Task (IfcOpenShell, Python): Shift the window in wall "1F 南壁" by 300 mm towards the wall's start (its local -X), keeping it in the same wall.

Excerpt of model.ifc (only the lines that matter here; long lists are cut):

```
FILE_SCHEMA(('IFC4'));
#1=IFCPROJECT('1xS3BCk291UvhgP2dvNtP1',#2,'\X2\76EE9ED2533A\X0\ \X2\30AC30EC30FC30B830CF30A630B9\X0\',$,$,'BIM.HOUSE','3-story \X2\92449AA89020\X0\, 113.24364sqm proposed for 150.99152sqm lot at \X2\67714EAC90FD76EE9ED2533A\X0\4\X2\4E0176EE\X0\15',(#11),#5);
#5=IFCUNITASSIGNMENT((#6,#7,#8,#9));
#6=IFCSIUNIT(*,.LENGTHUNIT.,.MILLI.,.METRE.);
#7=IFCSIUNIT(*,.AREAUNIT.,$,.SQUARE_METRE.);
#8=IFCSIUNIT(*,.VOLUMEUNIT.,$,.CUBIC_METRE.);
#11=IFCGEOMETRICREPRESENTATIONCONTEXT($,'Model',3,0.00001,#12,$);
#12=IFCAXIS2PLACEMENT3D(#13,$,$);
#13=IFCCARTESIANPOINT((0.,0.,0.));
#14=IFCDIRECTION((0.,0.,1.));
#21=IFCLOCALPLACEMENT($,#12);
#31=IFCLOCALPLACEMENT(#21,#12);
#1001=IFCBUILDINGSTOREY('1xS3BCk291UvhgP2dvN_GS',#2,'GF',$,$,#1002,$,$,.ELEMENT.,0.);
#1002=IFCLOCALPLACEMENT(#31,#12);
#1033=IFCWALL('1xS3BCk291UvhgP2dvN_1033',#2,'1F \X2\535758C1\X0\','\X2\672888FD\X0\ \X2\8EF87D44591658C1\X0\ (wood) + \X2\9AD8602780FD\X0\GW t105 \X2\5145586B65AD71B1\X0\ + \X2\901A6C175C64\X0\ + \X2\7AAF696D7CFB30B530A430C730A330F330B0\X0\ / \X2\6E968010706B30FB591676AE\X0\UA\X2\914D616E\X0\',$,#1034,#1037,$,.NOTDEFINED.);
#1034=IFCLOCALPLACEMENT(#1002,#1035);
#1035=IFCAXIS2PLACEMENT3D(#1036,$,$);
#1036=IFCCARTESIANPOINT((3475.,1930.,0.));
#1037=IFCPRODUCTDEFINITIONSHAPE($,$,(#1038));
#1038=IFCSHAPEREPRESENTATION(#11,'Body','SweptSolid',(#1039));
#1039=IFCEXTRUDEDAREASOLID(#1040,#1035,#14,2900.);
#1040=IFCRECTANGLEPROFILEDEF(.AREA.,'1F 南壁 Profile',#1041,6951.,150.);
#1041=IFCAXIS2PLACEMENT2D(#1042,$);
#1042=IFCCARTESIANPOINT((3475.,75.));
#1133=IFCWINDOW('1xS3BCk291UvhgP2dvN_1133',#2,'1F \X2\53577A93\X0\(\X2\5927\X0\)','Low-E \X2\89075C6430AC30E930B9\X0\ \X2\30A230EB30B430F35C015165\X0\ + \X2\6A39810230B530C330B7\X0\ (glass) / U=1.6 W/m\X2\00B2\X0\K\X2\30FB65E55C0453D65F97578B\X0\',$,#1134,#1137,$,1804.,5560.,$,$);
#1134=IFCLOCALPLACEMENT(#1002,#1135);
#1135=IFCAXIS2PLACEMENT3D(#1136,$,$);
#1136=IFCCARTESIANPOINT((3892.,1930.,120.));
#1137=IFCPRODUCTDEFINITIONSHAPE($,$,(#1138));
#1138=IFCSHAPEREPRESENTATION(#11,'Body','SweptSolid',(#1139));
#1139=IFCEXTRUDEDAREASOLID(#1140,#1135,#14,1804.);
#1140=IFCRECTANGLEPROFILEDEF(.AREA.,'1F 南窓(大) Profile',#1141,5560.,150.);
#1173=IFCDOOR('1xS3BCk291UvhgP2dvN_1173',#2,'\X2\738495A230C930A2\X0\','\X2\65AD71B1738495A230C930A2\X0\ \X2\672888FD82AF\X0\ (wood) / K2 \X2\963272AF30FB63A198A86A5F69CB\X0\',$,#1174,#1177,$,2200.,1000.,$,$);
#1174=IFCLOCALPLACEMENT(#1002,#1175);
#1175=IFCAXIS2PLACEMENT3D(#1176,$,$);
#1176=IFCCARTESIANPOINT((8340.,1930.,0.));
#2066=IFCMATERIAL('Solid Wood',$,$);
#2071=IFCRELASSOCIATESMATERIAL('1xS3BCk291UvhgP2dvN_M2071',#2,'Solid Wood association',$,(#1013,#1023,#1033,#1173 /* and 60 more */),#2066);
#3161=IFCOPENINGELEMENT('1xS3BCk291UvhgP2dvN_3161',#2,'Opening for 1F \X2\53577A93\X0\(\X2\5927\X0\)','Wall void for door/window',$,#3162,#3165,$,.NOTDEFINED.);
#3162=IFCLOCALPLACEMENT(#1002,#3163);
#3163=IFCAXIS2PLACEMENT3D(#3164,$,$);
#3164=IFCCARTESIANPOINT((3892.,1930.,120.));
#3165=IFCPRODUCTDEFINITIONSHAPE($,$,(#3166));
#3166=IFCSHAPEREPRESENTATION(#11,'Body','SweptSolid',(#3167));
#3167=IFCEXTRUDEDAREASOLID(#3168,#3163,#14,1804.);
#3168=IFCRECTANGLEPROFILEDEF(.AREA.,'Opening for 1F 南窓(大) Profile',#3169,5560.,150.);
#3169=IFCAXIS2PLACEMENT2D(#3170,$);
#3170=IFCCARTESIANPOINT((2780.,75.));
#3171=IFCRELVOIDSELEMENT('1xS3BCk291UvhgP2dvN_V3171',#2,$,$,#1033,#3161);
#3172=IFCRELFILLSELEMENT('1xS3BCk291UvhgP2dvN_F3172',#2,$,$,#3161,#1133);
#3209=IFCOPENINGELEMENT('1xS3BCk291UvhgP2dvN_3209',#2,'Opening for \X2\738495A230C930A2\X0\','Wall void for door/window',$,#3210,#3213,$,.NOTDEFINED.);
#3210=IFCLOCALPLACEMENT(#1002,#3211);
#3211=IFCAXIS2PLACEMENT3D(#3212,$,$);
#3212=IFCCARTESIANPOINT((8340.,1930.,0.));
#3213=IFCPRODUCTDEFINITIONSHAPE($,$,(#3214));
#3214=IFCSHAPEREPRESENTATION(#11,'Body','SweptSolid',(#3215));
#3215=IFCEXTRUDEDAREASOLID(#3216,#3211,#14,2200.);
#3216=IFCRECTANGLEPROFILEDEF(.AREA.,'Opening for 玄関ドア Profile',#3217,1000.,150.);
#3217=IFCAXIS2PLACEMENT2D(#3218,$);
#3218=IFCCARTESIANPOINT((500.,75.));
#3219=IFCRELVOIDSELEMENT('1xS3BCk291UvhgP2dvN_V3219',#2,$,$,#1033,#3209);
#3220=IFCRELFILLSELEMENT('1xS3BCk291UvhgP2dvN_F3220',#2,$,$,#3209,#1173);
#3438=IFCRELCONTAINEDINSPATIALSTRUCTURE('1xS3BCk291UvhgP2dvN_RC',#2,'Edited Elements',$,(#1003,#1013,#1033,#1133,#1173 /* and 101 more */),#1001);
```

```python
import ifcopenshell
import ifcopenshell.api.geometry
import ifcopenshell.util.placement
import ifcopenshell.util.unit

model = ifcopenshell.open("model.ifc")
unit_scale = ifcopenshell.util.unit.calculate_unit_scale(model)

window = model.by_guid("1xS3BCk291UvhgP2dvN_1133")
opening = window.FillsVoids[0].RelatingOpeningElement
wall = opening.VoidsElements[0].RelatingBuildingElement

wall_matrix = ifcopenshell.util.placement.get_local_placement(wall.ObjectPlacement)
shift = wall_matrix[:3, 0] * -0.3 / unit_scale
before = ifcopenshell.util.placement.get_local_placement(window.ObjectPlacement)[:3, 3].copy()

# The window is not placed relative to its opening, so move both.
for product in (opening, window):
    matrix = ifcopenshell.util.placement.get_local_placement(product.ObjectPlacement)
    matrix[:3, 3] += shift
    ifcopenshell.api.geometry.edit_object_placement(model, product=product, matrix=matrix, is_si=False)

after = ifcopenshell.util.placement.get_local_placement(window.ObjectPlacement)[:3, 3]
print("window moved by", (after - before).round(3) + 0.0)

model.write("model_rev.ifc")
```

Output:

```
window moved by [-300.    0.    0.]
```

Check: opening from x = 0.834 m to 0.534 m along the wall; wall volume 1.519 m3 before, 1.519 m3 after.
